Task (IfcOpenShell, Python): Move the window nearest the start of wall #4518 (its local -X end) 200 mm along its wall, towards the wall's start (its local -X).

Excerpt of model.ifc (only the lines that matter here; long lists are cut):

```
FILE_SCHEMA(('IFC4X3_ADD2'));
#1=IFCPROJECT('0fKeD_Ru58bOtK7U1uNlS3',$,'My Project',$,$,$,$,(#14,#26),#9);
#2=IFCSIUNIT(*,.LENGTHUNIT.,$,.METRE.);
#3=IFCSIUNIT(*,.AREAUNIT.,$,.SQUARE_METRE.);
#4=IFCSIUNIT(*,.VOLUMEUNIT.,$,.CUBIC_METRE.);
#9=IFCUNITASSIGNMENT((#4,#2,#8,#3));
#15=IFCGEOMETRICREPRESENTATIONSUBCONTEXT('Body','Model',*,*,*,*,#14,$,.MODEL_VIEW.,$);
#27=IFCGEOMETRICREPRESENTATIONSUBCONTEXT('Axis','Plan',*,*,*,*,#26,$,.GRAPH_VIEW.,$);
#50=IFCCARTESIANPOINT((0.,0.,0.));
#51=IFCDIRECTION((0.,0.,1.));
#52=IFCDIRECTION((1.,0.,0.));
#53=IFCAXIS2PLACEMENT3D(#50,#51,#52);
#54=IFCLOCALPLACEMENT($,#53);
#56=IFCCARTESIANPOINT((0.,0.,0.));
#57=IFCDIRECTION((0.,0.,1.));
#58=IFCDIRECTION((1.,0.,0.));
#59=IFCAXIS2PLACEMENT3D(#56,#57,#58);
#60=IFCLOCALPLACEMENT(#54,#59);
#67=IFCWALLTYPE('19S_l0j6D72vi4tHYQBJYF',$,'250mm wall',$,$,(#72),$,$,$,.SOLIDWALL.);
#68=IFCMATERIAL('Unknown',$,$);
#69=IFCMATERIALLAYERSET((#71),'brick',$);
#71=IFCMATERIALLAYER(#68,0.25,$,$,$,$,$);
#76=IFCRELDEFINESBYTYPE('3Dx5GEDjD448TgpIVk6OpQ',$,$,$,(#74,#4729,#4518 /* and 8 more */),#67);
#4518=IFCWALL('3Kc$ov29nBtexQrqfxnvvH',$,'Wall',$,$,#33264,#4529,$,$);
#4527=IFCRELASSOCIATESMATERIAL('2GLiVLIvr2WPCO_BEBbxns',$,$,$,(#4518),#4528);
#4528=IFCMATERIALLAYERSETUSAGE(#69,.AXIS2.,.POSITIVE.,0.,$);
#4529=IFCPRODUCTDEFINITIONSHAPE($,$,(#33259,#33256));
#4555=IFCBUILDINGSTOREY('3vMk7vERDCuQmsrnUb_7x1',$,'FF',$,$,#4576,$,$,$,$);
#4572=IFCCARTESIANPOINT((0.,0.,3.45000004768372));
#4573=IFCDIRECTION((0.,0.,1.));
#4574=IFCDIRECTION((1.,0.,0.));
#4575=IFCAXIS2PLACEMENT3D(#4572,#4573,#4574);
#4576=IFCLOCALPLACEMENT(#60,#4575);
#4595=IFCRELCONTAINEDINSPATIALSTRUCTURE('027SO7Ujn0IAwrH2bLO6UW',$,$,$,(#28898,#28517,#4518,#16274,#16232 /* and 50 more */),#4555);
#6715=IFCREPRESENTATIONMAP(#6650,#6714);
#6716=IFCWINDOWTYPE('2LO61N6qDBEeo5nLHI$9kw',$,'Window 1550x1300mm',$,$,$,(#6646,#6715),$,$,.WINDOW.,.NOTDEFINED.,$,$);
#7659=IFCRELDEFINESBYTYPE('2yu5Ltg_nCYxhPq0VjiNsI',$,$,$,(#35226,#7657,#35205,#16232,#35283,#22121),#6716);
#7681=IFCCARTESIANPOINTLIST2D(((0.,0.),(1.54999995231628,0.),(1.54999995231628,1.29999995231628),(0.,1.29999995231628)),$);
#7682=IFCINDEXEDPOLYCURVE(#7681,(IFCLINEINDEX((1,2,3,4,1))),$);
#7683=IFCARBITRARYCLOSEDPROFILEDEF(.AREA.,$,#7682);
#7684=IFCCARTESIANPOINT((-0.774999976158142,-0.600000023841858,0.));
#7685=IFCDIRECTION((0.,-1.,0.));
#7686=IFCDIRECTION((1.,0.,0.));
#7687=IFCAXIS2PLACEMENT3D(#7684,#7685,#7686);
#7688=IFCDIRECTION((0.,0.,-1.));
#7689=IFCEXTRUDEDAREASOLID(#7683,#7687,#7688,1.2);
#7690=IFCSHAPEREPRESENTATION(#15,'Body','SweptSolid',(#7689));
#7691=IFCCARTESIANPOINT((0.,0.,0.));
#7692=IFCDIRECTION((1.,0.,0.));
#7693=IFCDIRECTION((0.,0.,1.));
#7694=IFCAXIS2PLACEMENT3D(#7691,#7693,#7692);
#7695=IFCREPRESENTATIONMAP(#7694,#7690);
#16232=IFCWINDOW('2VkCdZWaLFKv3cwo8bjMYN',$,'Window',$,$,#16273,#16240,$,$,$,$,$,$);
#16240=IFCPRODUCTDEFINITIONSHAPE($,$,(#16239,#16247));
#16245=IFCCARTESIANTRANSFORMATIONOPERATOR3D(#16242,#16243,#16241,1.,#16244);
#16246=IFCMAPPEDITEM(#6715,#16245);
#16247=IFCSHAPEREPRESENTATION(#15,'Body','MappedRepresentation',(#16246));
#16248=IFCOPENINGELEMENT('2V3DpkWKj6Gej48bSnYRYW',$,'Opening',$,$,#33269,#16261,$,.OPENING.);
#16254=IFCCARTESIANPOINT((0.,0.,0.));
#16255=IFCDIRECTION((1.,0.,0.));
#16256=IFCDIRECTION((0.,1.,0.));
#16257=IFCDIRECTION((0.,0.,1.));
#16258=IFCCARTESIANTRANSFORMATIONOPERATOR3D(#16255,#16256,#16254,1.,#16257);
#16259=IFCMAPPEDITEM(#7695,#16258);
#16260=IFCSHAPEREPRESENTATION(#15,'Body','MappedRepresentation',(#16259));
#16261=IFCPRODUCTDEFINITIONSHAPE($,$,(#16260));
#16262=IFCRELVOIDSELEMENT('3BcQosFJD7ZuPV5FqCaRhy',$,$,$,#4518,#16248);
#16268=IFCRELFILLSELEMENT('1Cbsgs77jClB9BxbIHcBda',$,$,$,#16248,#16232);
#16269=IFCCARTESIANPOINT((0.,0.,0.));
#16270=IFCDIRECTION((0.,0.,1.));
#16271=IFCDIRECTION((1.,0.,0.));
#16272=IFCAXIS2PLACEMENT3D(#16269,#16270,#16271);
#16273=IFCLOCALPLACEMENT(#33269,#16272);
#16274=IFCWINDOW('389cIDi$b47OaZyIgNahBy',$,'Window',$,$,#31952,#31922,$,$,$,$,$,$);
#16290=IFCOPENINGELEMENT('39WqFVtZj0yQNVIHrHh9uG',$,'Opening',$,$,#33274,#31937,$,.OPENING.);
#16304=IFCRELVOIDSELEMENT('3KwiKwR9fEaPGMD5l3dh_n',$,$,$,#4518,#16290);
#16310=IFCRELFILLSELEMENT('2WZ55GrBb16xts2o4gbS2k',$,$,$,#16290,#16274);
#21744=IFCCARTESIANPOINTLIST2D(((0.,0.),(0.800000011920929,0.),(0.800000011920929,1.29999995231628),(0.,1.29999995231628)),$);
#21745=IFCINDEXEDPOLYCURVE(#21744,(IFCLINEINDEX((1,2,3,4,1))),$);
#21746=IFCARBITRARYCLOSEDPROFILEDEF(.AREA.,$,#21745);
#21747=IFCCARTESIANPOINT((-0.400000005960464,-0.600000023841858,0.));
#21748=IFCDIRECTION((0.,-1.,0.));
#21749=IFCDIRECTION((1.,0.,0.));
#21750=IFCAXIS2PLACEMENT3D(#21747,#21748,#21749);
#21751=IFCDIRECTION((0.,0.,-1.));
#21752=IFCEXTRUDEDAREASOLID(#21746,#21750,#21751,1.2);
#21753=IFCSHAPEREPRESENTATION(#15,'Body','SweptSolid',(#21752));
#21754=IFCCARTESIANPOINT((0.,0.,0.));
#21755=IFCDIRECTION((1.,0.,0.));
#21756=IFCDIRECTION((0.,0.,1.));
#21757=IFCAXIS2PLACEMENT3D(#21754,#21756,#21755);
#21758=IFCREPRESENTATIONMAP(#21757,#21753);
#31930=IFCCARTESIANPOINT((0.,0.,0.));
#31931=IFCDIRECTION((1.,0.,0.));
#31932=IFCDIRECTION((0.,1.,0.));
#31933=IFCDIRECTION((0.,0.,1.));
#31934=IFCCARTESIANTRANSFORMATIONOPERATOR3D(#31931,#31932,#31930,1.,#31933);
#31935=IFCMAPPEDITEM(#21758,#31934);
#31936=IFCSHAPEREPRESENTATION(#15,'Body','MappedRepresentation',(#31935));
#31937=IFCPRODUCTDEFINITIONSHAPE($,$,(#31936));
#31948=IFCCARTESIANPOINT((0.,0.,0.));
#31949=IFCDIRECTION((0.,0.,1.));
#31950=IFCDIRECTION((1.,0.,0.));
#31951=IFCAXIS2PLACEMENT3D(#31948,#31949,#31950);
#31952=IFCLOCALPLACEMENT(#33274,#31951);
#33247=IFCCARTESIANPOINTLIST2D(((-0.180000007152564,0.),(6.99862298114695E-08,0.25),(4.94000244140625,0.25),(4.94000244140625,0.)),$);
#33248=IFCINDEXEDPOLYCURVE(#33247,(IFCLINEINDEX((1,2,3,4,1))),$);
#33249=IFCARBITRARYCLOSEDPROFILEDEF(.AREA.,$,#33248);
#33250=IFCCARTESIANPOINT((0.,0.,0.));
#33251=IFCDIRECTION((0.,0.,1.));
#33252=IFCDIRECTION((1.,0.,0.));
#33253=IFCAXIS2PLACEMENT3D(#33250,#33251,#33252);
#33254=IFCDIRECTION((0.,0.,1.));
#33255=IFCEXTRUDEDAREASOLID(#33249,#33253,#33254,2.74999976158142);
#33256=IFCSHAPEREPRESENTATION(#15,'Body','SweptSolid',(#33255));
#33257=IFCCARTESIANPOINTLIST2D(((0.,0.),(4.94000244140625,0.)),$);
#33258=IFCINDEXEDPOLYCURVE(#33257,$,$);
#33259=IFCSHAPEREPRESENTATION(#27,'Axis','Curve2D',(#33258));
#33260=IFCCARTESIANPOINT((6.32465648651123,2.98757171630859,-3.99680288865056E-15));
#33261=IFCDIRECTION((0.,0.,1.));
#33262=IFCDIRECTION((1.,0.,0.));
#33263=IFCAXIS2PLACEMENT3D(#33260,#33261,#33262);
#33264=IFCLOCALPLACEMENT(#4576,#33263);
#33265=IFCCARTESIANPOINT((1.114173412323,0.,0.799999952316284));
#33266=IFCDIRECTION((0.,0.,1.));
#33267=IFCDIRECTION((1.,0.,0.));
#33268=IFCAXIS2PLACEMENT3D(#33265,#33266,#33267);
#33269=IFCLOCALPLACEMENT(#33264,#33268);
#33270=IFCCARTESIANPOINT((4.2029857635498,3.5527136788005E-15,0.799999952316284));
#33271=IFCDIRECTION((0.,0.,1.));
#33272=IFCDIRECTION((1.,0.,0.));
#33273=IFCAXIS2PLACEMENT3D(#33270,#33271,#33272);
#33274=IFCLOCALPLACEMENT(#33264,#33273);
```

```python
import ifcopenshell
import ifcopenshell.api.geometry
import ifcopenshell.util.placement
import ifcopenshell.util.unit

model = ifcopenshell.open("model.ifc")
unit_scale = ifcopenshell.util.unit.calculate_unit_scale(model)

window = model.by_guid("2VkCdZWaLFKv3cwo8bjMYN")
opening = window.FillsVoids[0].RelatingOpeningElement
wall = opening.VoidsElements[0].RelatingBuildingElement

wall_matrix = ifcopenshell.util.placement.get_local_placement(wall.ObjectPlacement)
shift = wall_matrix[:3, 0] * -0.2 / unit_scale
before = ifcopenshell.util.placement.get_local_placement(window.ObjectPlacement)[:3, 3].copy()

# The window is placed relative to its opening, so it follows when the opening moves.
matrix = ifcopenshell.util.placement.get_local_placement(opening.ObjectPlacement)
matrix[:3, 3] += shift
ifcopenshell.api.geometry.edit_object_placement(
    model, product=opening, matrix=matrix, is_si=False, should_transform_children=True
)

after = ifcopenshell.util.placement.get_local_placement(window.ObjectPlacement)[:3, 3]
print("window moved by", (after - before).round(3) + 0.0)

model.write("model_edited.ifc")
```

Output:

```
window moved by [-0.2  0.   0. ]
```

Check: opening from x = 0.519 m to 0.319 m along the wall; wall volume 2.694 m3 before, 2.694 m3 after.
